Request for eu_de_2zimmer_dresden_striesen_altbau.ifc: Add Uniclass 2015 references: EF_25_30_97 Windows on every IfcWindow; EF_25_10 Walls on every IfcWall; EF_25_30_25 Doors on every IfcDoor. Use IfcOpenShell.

First a look at what the model holds.

```python
import ifcopenshell

model = ifcopenshell.open("eu_de_2zimmer_dresden_striesen_altbau.ifc")
print(model.schema)
print("classifications:", [c.Name for c in model.by_type("IfcClassification")])
for ifc_class in ("IfcDoor", "IfcRoof", "IfcStair", "IfcWall", "IfcWindow"):
    print(ifc_class, len(model.by_type(ifc_class)))
```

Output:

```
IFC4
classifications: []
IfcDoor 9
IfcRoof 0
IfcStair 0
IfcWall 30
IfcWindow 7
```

```python
import ifcopenshell
import ifcopenshell.api.classification

model = ifcopenshell.open("eu_de_2zimmer_dresden_striesen_altbau.ifc")

system = ifcopenshell.api.classification.add_classification(model, classification="Uniclass 2015")

codes = {
    "IfcWindow": ("EF_25_30_97", "Windows"),
    "IfcWall": ("EF_25_10", "Walls"),
    "IfcDoor": ("EF_25_30_25", "Doors"),
}
for ifc_class, (code, name) in codes.items():
    products = model.by_type(ifc_class)
    ifcopenshell.api.classification.add_reference(
        model, products=products, classification=system, identification=code, name=name
    )
    print(code, len(products))

model.write("eu_de_2zimmer_dresden_striesen_altbau_v2.ifc")
```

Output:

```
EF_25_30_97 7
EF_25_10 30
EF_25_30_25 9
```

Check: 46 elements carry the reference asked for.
